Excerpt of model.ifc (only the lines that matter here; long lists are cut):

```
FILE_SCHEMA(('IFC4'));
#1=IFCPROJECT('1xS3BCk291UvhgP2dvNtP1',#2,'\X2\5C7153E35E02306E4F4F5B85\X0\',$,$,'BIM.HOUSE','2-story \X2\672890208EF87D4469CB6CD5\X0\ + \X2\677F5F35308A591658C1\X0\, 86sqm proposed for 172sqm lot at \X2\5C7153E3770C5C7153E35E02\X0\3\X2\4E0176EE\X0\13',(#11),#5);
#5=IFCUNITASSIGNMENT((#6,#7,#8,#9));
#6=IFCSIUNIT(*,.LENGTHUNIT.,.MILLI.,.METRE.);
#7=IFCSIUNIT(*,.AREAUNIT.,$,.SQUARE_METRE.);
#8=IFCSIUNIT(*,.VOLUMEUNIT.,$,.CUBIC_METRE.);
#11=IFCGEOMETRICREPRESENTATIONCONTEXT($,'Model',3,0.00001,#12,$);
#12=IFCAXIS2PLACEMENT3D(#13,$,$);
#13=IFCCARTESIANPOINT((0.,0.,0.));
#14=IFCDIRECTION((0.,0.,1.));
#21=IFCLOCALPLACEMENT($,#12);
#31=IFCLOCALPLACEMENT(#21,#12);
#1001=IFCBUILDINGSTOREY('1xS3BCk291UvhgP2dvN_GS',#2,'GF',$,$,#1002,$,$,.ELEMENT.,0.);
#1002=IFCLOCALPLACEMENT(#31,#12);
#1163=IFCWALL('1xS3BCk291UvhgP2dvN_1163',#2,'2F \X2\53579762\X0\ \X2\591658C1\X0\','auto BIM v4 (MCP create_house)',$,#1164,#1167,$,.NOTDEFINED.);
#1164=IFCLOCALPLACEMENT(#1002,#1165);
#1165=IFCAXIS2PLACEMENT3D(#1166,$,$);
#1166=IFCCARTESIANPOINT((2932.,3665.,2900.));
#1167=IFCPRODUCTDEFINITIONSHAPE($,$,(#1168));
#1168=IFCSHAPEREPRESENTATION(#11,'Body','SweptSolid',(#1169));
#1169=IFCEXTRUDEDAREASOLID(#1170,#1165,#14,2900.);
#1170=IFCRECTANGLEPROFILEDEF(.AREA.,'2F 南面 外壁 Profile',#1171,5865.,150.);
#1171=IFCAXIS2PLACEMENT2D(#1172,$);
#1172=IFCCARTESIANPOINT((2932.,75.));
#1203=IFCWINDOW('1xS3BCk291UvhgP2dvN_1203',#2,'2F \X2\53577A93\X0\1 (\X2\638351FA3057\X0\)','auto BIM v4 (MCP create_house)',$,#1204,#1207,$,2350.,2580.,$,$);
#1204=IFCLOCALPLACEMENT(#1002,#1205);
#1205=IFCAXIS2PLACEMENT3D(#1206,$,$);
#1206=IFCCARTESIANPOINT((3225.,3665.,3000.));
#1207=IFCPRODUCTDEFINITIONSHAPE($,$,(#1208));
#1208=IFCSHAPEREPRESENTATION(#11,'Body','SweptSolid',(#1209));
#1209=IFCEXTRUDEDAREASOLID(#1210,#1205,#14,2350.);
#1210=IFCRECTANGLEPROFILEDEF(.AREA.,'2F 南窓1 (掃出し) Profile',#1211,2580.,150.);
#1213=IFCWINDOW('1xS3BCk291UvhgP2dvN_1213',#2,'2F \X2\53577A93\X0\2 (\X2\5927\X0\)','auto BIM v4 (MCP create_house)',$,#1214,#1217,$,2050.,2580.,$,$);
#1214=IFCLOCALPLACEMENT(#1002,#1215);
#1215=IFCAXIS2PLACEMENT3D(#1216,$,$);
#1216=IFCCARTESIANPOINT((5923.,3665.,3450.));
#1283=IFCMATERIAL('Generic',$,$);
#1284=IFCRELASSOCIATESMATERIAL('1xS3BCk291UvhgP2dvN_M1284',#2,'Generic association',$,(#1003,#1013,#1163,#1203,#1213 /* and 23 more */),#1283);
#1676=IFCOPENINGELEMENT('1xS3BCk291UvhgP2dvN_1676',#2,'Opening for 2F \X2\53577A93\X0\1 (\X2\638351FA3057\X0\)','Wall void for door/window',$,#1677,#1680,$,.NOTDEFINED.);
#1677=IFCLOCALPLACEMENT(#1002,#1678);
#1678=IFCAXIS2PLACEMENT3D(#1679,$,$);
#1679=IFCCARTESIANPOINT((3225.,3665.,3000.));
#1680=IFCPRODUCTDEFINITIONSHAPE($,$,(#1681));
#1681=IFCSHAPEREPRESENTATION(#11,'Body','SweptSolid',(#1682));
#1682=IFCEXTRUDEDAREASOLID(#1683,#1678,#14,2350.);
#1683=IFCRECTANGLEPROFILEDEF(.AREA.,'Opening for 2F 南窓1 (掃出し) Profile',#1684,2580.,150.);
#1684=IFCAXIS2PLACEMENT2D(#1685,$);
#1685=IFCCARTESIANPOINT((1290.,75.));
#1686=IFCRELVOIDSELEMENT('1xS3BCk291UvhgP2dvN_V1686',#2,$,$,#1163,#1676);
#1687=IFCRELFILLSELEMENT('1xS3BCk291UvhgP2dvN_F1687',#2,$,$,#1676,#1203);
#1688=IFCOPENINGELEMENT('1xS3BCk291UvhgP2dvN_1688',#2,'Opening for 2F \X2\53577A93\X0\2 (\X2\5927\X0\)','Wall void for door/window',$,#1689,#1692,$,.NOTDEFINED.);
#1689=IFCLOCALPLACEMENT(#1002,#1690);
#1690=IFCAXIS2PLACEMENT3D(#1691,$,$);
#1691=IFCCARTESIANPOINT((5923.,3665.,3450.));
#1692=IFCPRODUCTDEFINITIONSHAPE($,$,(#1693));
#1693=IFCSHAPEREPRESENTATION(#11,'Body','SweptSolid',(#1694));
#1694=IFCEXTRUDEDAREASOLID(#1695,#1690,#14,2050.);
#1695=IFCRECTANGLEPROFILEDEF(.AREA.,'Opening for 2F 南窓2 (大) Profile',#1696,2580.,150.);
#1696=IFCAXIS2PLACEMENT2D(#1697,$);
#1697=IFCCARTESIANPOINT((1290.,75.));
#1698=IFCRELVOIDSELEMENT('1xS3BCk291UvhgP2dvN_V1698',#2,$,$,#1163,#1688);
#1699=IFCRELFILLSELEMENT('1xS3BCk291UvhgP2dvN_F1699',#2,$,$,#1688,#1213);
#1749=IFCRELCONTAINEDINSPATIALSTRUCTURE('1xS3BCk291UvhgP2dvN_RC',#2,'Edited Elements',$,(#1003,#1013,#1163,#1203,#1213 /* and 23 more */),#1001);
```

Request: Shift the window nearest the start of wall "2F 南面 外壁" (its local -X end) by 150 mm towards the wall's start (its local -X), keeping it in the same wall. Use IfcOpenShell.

```python
import ifcopenshell
import ifcopenshell.api.geometry
import ifcopenshell.util.placement
import ifcopenshell.util.unit

model = ifcopenshell.open("model.ifc")
unit_scale = ifcopenshell.util.unit.calculate_unit_scale(model)

window = model.by_guid("1xS3BCk291UvhgP2dvN_1203")
opening = window.FillsVoids[0].RelatingOpeningElement
wall = opening.VoidsElements[0].RelatingBuildingElement

wall_matrix = ifcopenshell.util.placement.get_local_placement(wall.ObjectPlacement)
shift = wall_matrix[:3, 0] * -0.15 / unit_scale
before = ifcopenshell.util.placement.get_local_placement(window.ObjectPlacement)[:3, 3].copy()

# The window is not placed relative to its opening, so move both.
for product in (opening, window):
    matrix = ifcopenshell.util.placement.get_local_placement(product.ObjectPlacement)
    matrix[:3, 3] += shift
    ifcopenshell.api.geometry.edit_object_placement(model, product=product, matrix=matrix, is_si=False)

after = ifcopenshell.util.placement.get_local_placement(window.ObjectPlacement)[:3, 3]
print("window moved by", (after - before).round(3) + 0.0)

model.write("model-out.ifc")
```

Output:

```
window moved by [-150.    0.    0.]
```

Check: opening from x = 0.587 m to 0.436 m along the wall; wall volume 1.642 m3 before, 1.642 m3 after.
